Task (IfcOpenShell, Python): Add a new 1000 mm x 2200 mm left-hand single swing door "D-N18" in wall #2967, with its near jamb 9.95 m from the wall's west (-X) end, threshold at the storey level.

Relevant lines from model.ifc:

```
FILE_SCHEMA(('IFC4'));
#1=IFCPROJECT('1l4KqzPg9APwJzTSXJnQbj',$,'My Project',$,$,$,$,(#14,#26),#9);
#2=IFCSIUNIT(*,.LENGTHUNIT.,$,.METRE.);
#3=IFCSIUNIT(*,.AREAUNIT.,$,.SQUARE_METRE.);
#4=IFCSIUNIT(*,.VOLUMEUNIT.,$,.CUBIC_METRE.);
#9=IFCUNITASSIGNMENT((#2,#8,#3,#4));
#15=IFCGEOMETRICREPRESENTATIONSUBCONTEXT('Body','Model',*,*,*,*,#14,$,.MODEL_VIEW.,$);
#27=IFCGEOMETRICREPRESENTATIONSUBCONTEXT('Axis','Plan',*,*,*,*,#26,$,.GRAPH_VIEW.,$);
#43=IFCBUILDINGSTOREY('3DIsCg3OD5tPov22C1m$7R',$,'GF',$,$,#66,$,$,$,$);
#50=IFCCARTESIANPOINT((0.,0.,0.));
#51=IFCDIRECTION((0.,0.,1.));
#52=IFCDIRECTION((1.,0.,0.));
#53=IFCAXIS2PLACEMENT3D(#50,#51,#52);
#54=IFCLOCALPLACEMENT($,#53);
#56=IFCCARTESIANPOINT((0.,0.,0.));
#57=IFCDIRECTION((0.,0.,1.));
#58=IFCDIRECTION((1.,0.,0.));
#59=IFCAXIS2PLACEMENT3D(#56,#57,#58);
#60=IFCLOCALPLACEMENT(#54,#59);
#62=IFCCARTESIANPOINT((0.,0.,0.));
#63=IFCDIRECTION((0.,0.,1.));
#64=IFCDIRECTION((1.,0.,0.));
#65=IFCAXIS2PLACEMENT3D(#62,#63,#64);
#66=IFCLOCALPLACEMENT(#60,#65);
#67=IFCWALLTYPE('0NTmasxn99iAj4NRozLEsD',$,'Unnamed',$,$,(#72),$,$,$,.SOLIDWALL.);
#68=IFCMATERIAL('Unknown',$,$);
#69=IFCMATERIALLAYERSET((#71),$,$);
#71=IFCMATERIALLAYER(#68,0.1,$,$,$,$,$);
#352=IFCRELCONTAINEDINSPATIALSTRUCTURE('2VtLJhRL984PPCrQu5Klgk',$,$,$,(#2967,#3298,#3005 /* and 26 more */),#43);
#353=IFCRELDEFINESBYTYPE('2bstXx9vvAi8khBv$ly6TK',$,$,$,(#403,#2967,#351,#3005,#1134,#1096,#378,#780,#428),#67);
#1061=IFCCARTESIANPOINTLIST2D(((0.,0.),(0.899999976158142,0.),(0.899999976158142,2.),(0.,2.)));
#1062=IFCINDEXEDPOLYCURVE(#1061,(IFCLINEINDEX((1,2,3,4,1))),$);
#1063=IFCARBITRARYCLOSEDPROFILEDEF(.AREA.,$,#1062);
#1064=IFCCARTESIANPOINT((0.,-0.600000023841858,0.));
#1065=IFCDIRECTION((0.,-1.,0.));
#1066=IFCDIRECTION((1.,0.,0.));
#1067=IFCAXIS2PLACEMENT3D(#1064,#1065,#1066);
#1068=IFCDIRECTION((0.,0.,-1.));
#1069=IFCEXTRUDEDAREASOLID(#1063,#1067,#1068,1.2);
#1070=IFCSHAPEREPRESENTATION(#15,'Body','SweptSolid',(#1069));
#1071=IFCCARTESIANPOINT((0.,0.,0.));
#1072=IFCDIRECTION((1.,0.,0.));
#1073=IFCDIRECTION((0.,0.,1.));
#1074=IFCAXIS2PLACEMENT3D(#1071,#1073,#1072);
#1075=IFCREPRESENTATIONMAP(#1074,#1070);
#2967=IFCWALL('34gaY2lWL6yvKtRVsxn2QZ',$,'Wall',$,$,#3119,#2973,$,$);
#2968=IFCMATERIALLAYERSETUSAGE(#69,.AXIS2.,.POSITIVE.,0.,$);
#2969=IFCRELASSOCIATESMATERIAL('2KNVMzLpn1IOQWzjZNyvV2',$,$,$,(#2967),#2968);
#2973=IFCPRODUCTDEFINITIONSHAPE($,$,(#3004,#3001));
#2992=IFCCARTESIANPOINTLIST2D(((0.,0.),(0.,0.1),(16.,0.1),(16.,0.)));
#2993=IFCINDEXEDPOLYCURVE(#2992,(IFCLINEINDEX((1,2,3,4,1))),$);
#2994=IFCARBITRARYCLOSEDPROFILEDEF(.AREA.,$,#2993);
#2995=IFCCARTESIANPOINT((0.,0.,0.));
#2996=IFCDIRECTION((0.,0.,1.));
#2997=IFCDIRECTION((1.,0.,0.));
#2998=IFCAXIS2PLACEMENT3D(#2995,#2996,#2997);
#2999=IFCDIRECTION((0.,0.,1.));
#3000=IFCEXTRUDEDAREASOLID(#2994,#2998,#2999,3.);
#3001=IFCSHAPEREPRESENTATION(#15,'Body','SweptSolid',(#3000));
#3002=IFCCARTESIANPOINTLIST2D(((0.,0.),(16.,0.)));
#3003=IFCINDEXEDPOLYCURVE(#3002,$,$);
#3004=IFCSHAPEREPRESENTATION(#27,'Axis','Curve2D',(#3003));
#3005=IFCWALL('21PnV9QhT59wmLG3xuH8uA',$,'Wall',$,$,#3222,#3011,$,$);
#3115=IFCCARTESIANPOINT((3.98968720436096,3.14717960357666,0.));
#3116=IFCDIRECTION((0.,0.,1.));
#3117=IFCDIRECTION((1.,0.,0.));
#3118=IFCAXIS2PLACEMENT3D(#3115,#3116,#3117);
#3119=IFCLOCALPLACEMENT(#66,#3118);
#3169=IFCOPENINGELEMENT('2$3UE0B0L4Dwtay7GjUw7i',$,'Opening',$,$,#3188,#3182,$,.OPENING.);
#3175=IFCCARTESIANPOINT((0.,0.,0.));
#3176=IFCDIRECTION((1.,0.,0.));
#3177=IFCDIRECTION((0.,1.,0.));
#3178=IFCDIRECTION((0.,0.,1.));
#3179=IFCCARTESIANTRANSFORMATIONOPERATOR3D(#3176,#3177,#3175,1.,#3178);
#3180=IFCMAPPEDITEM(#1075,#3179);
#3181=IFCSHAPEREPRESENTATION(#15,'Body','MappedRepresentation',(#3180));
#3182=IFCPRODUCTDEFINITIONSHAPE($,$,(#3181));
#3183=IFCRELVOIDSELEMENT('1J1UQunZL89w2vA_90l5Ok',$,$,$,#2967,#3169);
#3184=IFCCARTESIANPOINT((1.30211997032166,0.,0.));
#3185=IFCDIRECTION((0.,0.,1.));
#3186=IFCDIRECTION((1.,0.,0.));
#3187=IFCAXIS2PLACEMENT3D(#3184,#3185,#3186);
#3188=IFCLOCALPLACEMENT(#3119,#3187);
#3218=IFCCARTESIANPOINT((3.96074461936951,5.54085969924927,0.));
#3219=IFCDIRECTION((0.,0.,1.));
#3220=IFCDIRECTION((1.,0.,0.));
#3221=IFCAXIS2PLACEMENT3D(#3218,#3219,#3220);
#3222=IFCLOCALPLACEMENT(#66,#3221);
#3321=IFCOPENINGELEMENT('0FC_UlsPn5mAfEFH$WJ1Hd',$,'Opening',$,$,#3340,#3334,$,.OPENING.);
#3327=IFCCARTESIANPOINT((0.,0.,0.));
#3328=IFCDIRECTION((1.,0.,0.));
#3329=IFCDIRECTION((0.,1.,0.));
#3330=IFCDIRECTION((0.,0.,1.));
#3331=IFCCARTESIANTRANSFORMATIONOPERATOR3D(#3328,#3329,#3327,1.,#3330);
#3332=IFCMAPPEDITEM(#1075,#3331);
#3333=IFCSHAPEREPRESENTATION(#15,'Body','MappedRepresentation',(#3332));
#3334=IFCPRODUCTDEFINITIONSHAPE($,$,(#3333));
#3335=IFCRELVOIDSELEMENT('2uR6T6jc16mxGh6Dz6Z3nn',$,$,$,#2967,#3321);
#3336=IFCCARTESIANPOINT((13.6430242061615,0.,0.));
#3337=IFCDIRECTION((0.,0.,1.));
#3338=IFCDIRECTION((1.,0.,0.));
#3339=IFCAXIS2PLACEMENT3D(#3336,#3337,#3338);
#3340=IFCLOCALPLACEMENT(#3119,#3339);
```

```python
import numpy as np
import ifcopenshell
import ifcopenshell.api.feature
import ifcopenshell.api.geometry
import ifcopenshell.api.root
import ifcopenshell.api.spatial
import ifcopenshell.geom
import ifcopenshell.util.element
import ifcopenshell.util.placement
import ifcopenshell.util.representation
import ifcopenshell.util.shape
import ifcopenshell.util.unit

model = ifcopenshell.open("model.ifc")
unit_scale = ifcopenshell.util.unit.calculate_unit_scale(model)
settings = ifcopenshell.geom.settings()


def volume(element):
    """Net volume in cubic metres, openings subtracted."""
    shape = ifcopenshell.geom.create_shape(settings, element)
    return ifcopenshell.util.shape.get_volume(shape.geometry)


wall = model.by_guid("34gaY2lWL6yvKtRVsxn2QZ")
storey = ifcopenshell.util.element.get_container(wall, ifc_class="IfcBuildingStorey")
context = ifcopenshell.util.representation.get_context(model, "Model", "Body", "MODEL_VIEW")
before = volume(wall)

width, height, from_end, sill = 1, 2.2, 9.95, 0.0  # metres

# The wall runs along its own X axis, and the end named is its -X end.
wall_shape = ifcopenshell.geom.create_shape(settings, wall)
x, y, z = ifcopenshell.util.shape.get_vertices(wall_shape.geometry).T
start = x.min() + from_end
face, thickness = float(y.min()), float(y.max() - y.min())
wall_matrix = ifcopenshell.util.placement.get_local_placement(wall.ObjectPlacement)
level = ifcopenshell.util.placement.get_local_placement(storey.ObjectPlacement)[2, 3]


def in_wall(x, y):
    """Placement at x, y metres in the wall's axes, at sill height."""
    matrix = wall_matrix.copy()
    matrix[:, 3] = wall_matrix @ np.array([x / unit_scale, y / unit_scale, 0.0, 1.0])
    matrix[2, 3] = level + sill / unit_scale
    return matrix


# Opening: a box that overshoots both wall faces by 50 mm.
opening = ifcopenshell.api.root.create_entity(model, ifc_class="IfcOpeningElement", predefined_type="OPENING")
box = ifcopenshell.api.geometry.add_wall_representation(
    model, context=context, length=width, height=height, thickness=thickness + 0.1
)
ifcopenshell.api.geometry.assign_representation(model, product=opening, representation=box)
ifcopenshell.api.geometry.edit_object_placement(model, product=opening, matrix=in_wall(start, face - 0.05), is_si=False)
ifcopenshell.api.feature.add_feature(model, feature=opening, element=wall)

door = ifcopenshell.api.root.create_entity(model, ifc_class="IfcDoor", name="D-N18", predefined_type="DOOR")
door.OverallWidth, door.OverallHeight = width / unit_scale, height / unit_scale
door.OperationType = "SINGLE_SWING_LEFT"
body = ifcopenshell.api.geometry.add_door_representation(
    model,
    context=context,
    overall_width=door.OverallWidth,
    overall_height=door.OverallHeight,
    operation_type="SINGLE_SWING_LEFT",
    lining_properties={"LiningDepth": thickness / unit_scale, "ThresholdDepth": thickness / unit_scale},
)
ifcopenshell.api.geometry.assign_representation(model, product=door, representation=body)
ifcopenshell.api.spatial.assign_container(model, products=[door], relating_structure=storey)
ifcopenshell.api.feature.add_filling(model, opening=opening, element=door)

# The lining spans the wall, so the door starts at the wall face.
ifcopenshell.api.geometry.edit_object_placement(model, product=door, matrix=in_wall(start, face), is_si=False)

after = volume(wall)

print(f"wall volume {before:.3f} -> {after:.3f} m3")

model.write("model_rev.ifc")
```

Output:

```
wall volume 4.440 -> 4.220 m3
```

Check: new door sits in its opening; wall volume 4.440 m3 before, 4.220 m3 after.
